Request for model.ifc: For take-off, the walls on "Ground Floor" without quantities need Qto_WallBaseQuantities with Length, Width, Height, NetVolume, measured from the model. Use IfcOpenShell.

First a look at what the model holds.

```python
import ifcopenshell
import ifcopenshell.util.element
import ifcopenshell.util.unit

model = ifcopenshell.open("model.ifc")
print(model.schema)
for unit_type in ("LENGTHUNIT", "AREAUNIT", "VOLUMEUNIT"):
    print(unit_type, ifcopenshell.util.unit.calculate_unit_scale(model, unit_type))
storey = next(s for s in model.by_type("IfcBuildingStorey") if s.Name == "Ground Floor")
walls = [e for e in ifcopenshell.util.element.get_decomposition(storey) if e.is_a("IfcWall")]
for e in sorted(walls, key=lambda e: e.id()):
    print(e.id(), e.is_a(), e.Name, list(ifcopenshell.util.element.get_psets(e, qtos_only=True)), sep=" | ")
```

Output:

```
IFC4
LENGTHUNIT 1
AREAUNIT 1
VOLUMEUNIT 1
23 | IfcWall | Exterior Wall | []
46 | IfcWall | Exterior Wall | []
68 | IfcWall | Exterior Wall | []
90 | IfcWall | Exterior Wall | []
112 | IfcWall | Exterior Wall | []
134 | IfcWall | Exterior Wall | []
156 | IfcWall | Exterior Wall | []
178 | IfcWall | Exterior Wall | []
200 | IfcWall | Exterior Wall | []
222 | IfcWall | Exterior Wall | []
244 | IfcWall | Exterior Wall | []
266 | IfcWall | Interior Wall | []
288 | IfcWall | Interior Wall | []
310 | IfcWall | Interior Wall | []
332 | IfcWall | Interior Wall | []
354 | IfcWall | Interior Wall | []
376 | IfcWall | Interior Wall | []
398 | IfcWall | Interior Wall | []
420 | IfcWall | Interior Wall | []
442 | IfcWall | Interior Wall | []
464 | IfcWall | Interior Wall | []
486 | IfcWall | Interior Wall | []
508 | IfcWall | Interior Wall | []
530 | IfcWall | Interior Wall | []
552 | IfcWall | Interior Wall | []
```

```python
import ifcopenshell
import ifcopenshell.api.pset
import ifcopenshell.geom
import ifcopenshell.util.element
import ifcopenshell.util.shape
import ifcopenshell.util.unit

model = ifcopenshell.open("model.ifc")
unit_scale = ifcopenshell.util.unit.calculate_unit_scale(model)
volume_scale = ifcopenshell.util.unit.calculate_unit_scale(model, "VOLUMEUNIT")
settings = ifcopenshell.geom.settings()

storey = next(s for s in model.by_type("IfcBuildingStorey") if s.Name == "Ground Floor")
walls = [e for e in ifcopenshell.util.element.get_decomposition(storey) if e.is_a("IfcWall")]

for e in sorted(walls, key=lambda e: e.id()):
    if ifcopenshell.util.element.get_psets(e, qtos_only=True, should_inherit=False):
        continue
    # Geometry comes back in metres, in the element's own axes.
    shape = ifcopenshell.geom.create_shape(settings, e)
    values = {
        "Length": ifcopenshell.util.shape.get_x(shape.geometry) / unit_scale,
        "Width": ifcopenshell.util.shape.get_y(shape.geometry) / unit_scale,
        "Height": ifcopenshell.util.shape.get_z(shape.geometry) / unit_scale,
        "NetVolume": ifcopenshell.util.shape.get_volume(shape.geometry) / volume_scale,
    }
    qto = ifcopenshell.api.pset.add_qto(model, product=e, name="Qto_WallBaseQuantities")
    ifcopenshell.api.pset.edit_qto(model, qto=qto, properties=values)
    print(e.id(), {k: round(v, 3) for k, v in values.items()})

model.write("model-out.ifc")
```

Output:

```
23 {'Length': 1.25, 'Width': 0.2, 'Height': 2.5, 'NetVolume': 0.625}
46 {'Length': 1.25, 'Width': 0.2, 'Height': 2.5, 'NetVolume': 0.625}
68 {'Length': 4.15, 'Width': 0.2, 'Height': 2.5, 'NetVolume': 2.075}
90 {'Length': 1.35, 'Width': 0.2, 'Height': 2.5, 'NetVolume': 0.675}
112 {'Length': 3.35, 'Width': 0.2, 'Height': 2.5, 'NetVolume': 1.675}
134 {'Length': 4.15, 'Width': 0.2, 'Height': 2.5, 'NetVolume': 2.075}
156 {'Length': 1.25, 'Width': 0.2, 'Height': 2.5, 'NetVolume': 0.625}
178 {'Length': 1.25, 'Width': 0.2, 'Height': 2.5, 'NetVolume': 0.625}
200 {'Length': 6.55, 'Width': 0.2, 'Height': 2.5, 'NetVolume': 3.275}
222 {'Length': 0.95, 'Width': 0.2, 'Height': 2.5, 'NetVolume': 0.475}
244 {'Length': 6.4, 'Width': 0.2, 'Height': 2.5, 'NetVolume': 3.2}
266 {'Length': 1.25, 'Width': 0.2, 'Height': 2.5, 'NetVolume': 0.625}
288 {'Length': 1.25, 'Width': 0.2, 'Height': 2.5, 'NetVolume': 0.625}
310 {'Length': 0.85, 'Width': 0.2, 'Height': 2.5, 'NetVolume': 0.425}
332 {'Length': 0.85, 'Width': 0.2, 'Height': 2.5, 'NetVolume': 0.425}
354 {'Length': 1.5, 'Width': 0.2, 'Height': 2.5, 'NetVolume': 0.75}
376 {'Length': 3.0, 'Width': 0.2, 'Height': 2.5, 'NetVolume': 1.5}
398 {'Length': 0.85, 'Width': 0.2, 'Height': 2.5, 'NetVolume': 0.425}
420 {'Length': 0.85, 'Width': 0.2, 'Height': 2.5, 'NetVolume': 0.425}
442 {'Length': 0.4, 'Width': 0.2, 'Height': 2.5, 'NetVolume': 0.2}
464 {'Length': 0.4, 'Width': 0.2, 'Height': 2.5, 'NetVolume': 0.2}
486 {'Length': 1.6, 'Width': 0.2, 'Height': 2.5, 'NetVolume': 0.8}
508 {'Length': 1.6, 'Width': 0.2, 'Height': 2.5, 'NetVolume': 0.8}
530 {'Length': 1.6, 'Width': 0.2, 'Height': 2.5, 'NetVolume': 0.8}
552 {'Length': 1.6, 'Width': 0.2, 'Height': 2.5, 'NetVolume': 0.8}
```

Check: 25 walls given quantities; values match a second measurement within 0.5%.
